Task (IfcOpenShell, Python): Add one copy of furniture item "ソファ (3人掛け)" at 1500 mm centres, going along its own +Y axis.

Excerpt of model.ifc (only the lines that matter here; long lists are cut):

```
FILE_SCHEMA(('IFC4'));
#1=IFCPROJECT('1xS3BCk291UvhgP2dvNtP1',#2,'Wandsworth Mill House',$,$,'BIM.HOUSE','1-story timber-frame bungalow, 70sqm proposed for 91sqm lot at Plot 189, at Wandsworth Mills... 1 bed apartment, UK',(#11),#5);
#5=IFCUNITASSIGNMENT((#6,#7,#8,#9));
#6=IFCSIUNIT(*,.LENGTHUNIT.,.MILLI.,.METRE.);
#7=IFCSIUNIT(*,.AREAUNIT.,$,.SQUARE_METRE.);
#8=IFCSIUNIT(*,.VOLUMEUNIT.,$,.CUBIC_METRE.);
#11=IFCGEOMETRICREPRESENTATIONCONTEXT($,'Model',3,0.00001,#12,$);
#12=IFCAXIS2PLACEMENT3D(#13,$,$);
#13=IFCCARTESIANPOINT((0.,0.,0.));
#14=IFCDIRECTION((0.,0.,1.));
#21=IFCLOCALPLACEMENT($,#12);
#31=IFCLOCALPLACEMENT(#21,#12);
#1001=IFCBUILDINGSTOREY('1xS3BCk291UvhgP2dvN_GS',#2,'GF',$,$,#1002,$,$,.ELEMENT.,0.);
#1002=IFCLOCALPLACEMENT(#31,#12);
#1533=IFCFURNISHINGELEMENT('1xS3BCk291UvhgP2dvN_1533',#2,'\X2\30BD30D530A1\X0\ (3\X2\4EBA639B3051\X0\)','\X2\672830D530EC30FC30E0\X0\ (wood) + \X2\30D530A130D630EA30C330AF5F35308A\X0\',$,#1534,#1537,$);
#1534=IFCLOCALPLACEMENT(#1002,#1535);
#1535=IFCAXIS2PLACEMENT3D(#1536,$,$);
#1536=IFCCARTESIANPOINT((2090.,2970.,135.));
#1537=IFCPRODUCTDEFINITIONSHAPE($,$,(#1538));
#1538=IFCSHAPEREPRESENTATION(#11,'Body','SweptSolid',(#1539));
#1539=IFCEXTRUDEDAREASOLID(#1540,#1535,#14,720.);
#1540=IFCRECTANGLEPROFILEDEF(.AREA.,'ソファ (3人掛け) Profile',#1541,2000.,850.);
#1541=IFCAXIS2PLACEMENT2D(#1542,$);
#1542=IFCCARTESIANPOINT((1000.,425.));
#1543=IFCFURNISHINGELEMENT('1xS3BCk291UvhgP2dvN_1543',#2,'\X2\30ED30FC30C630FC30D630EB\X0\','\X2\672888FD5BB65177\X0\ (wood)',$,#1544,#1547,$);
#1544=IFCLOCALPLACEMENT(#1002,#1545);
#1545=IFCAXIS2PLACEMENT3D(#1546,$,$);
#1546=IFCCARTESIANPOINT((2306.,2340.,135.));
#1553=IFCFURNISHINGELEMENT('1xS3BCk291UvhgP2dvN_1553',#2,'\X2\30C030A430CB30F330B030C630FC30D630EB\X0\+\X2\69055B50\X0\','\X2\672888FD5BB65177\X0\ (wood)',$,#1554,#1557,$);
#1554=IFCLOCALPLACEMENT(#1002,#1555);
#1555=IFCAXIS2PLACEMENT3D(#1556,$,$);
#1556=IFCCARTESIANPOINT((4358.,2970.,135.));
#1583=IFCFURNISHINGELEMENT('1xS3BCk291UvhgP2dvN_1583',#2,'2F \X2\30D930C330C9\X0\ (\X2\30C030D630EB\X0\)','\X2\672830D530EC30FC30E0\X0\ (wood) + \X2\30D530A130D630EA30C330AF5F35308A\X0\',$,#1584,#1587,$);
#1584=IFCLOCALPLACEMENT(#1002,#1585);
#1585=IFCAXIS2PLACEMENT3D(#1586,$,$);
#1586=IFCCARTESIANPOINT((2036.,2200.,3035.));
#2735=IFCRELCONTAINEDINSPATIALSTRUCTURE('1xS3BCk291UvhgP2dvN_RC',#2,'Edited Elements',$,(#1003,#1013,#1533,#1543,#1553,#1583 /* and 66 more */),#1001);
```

```python
import ifcopenshell
import ifcopenshell.api.geometry
import ifcopenshell.api.root
import ifcopenshell.util.element
import ifcopenshell.util.placement
import ifcopenshell.util.unit

model = ifcopenshell.open("model.ifc")
unit_scale = ifcopenshell.util.unit.calculate_unit_scale(model)


def reuse_history(source, copy):
    """copy_class also copies each property set's owner history, people and application; keep the originals."""
    for rel in copy.IsDefinedBy:
        if rel.is_a("IfcRelDefinesByProperties") and (history := rel.RelatingPropertyDefinition.OwnerHistory):
            rel.RelatingPropertyDefinition.OwnerHistory = source.OwnerHistory
            ifcopenshell.util.element.remove_deep2(model, history)


source = model.by_guid("1xS3BCk291UvhgP2dvN_1533")
base = ifcopenshell.util.placement.get_local_placement(source.ObjectPlacement)
step = base[:3, 1] * 1.5 / unit_scale

for i in range(1, 2):
    copy = ifcopenshell.api.root.copy_class(model, product=source)
    copy.Representation = ifcopenshell.util.element.copy_deep(
        model, source.Representation, exclude=["IfcGeometricRepresentationContext", "IfcRepresentationMap"]
    )
    reuse_history(source, copy)
    matrix = base.copy()
    matrix[:3, 3] += i * step
    print("added at", matrix[:3, 3].round(3) + 0.0)
    ifcopenshell.api.geometry.edit_object_placement(model, product=copy, matrix=matrix, is_si=False)

model.write("model_edited.ifc")
```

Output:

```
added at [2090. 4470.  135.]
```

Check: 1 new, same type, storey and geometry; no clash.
